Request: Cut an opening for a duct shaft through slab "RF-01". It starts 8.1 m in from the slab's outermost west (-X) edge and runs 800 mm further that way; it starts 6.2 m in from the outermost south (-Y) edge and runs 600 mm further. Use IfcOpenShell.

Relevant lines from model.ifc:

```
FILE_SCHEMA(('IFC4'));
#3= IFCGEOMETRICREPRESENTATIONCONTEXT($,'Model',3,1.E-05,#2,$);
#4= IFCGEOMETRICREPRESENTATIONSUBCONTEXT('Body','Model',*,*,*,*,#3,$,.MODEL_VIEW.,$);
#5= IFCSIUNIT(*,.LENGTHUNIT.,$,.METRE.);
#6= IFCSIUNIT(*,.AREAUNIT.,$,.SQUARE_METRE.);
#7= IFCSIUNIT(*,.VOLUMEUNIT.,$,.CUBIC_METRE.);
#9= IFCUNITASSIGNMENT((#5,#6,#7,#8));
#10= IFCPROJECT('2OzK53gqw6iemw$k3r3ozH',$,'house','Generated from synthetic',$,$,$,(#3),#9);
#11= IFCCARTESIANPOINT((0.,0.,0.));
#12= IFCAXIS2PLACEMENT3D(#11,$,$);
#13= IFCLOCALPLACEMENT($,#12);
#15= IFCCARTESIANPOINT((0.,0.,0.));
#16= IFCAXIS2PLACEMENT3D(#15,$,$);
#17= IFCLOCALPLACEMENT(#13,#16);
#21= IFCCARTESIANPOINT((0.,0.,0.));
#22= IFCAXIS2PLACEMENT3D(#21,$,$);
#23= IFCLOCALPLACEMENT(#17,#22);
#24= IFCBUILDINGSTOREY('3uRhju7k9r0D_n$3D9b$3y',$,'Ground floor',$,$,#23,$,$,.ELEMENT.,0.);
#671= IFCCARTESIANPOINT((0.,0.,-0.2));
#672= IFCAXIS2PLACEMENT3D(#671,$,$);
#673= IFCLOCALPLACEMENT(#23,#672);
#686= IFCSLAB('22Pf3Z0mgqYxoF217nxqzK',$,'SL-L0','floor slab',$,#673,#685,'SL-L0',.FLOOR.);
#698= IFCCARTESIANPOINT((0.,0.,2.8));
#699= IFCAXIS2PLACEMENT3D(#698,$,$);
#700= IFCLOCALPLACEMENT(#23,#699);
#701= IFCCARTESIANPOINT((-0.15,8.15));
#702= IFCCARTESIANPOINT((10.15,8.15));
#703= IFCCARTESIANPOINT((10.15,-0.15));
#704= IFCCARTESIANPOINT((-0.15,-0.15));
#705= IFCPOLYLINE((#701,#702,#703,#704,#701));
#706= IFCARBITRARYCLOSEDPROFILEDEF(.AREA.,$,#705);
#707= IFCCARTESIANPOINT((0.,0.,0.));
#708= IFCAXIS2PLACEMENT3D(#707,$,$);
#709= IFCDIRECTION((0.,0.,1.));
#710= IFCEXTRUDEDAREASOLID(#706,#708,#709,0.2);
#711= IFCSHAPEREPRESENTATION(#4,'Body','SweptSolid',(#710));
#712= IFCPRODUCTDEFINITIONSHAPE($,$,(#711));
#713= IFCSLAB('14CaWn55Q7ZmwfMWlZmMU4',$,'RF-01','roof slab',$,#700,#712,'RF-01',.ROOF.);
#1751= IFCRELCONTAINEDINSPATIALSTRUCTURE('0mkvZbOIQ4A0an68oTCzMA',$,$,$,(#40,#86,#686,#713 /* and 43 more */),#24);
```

```python
import numpy as np
import ifcopenshell
import ifcopenshell.api.feature
import ifcopenshell.api.geometry
import ifcopenshell.api.root
import ifcopenshell.geom
import ifcopenshell.util.placement
import ifcopenshell.util.representation
import ifcopenshell.util.shape
import ifcopenshell.util.unit

model = ifcopenshell.open("model.ifc")
unit_scale = ifcopenshell.util.unit.calculate_unit_scale(model)
settings = ifcopenshell.geom.settings()


def volume(element):
    """Net volume in cubic metres, openings subtracted."""
    shape = ifcopenshell.geom.create_shape(settings, element)
    return ifcopenshell.util.shape.get_volume(shape.geometry)


slab = model.by_id(713)
before = volume(slab)

# Extent in the slab's own axes, in metres. The edges named are its -X and -Y sides.
slab_shape = ifcopenshell.geom.create_shape(settings, slab)
vertices = ifcopenshell.util.shape.get_vertices(slab_shape.geometry)
x_min, y_min, bottom = vertices.min(axis=0)
top = vertices[:, 2].max()

opening = ifcopenshell.api.root.create_entity(model, ifc_class="IfcOpeningElement", name="Duct shaft opening", predefined_type="OPENING")
context = ifcopenshell.util.representation.get_context(model, "Model", "Body", "MODEL_VIEW")
width, depth = 0.8, 0.6
outline = [(0.0, 0.0), (width, 0.0), (width, depth), (0.0, depth), (0.0, 0.0)]
# Overshoot both faces by 50 mm so the cut is clean.
shape = ifcopenshell.api.geometry.add_slab_representation(
    model, context=context, depth=top - bottom + 0.1, polyline=outline
)
ifcopenshell.api.geometry.assign_representation(model, product=opening, representation=shape)

matrix = ifcopenshell.util.placement.get_local_placement(slab.ObjectPlacement)
matrix[:, 3] = matrix @ np.append(np.array([x_min + 8.1, y_min + 6.2, bottom - 0.05]) / unit_scale, 1.0)
ifcopenshell.api.geometry.edit_object_placement(model, product=opening, matrix=matrix, is_si=False)
ifcopenshell.api.feature.add_feature(model, feature=opening, element=slab)

after = volume(slab)

print(f"slab volume {before:.3f} -> {after:.3f} m3")

model.write("model_rev.ifc")
```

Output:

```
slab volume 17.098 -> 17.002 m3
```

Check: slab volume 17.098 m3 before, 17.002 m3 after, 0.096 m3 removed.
